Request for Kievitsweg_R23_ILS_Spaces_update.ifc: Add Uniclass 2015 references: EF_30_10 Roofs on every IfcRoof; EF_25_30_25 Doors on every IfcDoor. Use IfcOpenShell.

First a look at what the model holds.

```python
import ifcopenshell

model = ifcopenshell.open("Kievitsweg_R23_ILS_Spaces_update.ifc")
print(model.schema)
print("classifications:", [c.Name for c in model.by_type("IfcClassification")])
for ifc_class in ("IfcDoor", "IfcRoof", "IfcStair", "IfcWall", "IfcWindow"):
    print(ifc_class, len(model.by_type(ifc_class)))
```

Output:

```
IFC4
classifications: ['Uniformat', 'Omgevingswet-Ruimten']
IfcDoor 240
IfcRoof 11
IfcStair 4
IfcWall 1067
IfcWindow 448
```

```python
import ifcopenshell
import ifcopenshell.api.classification

model = ifcopenshell.open("Kievitsweg_R23_ILS_Spaces_update.ifc")

system = ifcopenshell.api.classification.add_classification(model, classification="Uniclass 2015")

codes = {
    "IfcRoof": ("EF_30_10", "Roofs"),
    "IfcDoor": ("EF_25_30_25", "Doors"),
}
for ifc_class, (code, name) in codes.items():
    products = model.by_type(ifc_class)
    ifcopenshell.api.classification.add_reference(
        model, products=products, classification=system, identification=code, name=name
    )
    print(code, len(products))

model.write("Kievitsweg_R23_ILS_Spaces_update_edited.ifc")
```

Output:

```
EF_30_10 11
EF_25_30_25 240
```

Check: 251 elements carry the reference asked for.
